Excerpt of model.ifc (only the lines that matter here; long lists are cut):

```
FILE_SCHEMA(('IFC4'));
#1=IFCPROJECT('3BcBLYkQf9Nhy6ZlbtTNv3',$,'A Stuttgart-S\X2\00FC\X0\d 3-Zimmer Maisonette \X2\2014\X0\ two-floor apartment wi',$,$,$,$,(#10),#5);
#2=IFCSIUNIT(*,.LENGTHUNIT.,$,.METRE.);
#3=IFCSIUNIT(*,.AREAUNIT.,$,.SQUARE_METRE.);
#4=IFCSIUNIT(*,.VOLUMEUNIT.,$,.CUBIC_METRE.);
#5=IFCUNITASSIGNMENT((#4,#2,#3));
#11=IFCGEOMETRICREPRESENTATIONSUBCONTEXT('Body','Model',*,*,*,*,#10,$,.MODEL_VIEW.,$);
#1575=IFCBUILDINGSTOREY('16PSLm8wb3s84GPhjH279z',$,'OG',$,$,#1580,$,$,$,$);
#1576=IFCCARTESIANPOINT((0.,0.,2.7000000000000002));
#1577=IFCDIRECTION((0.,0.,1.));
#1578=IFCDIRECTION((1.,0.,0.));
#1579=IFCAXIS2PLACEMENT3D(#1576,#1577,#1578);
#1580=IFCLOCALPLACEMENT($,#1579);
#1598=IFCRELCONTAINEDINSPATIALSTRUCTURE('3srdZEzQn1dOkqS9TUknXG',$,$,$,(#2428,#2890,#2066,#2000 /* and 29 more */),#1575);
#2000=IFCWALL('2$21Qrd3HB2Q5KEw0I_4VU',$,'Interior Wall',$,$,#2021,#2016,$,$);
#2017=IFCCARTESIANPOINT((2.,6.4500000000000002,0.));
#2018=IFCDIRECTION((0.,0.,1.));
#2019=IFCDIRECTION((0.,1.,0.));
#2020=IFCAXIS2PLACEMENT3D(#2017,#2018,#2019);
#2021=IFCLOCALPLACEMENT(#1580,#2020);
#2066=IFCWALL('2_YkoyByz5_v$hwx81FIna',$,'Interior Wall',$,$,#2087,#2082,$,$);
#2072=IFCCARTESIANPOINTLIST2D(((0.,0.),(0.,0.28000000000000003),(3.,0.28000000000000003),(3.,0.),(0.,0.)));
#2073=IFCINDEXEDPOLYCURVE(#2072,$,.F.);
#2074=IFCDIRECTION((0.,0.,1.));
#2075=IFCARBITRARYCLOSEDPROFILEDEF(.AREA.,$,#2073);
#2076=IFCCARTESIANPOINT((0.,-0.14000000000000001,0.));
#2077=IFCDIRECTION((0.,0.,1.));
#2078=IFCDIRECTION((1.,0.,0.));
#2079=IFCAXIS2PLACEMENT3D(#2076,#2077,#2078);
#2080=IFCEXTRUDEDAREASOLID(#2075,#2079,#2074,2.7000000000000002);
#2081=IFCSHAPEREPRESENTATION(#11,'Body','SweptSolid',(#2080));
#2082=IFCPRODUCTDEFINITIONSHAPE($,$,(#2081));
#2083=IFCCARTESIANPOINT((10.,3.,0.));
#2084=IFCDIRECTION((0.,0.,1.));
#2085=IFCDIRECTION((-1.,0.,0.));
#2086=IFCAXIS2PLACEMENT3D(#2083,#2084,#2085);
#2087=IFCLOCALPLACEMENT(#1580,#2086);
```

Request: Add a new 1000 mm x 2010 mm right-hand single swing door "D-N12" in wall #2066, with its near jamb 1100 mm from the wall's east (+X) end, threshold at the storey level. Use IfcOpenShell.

```python
import numpy as np
import ifcopenshell
import ifcopenshell.api.feature
import ifcopenshell.api.geometry
import ifcopenshell.api.root
import ifcopenshell.api.spatial
import ifcopenshell.geom
import ifcopenshell.util.element
import ifcopenshell.util.placement
import ifcopenshell.util.representation
import ifcopenshell.util.shape
import ifcopenshell.util.unit

model = ifcopenshell.open("model.ifc")
unit_scale = ifcopenshell.util.unit.calculate_unit_scale(model)
settings = ifcopenshell.geom.settings()


def volume(element):
    """Net volume in cubic metres, openings subtracted."""
    shape = ifcopenshell.geom.create_shape(settings, element)
    return ifcopenshell.util.shape.get_volume(shape.geometry)


wall = model.by_id(2066)
storey = ifcopenshell.util.element.get_container(wall, ifc_class="IfcBuildingStorey")
context = ifcopenshell.util.representation.get_context(model, "Model", "Body", "MODEL_VIEW")
before = volume(wall)

width, height, from_end, sill = 1, 2.01, 1.1, 0.0  # metres

# The wall runs along its own X axis, and the end named is its -X end.
wall_shape = ifcopenshell.geom.create_shape(settings, wall)
x, y, z = ifcopenshell.util.shape.get_vertices(wall_shape.geometry).T
start = x.min() + from_end
face, thickness = float(y.min()), float(y.max() - y.min())
wall_matrix = ifcopenshell.util.placement.get_local_placement(wall.ObjectPlacement)
level = ifcopenshell.util.placement.get_local_placement(storey.ObjectPlacement)[2, 3]


def in_wall(x, y):
    """Placement at x, y metres in the wall's axes, at sill height."""
    matrix = wall_matrix.copy()
    matrix[:, 3] = wall_matrix @ np.array([x / unit_scale, y / unit_scale, 0.0, 1.0])
    matrix[2, 3] = level + sill / unit_scale
    return matrix


# Opening: a box that overshoots both wall faces by 50 mm.
opening = ifcopenshell.api.root.create_entity(model, ifc_class="IfcOpeningElement", predefined_type="OPENING")
box = ifcopenshell.api.geometry.add_wall_representation(
    model, context=context, length=width, height=height, thickness=thickness + 0.1
)
ifcopenshell.api.geometry.assign_representation(model, product=opening, representation=box)
ifcopenshell.api.geometry.edit_object_placement(model, product=opening, matrix=in_wall(start, face - 0.05), is_si=False)
ifcopenshell.api.feature.add_feature(model, feature=opening, element=wall)

door = ifcopenshell.api.root.create_entity(model, ifc_class="IfcDoor", name="D-N12", predefined_type="DOOR")
door.OverallWidth, door.OverallHeight = width / unit_scale, height / unit_scale
door.OperationType = "SINGLE_SWING_RIGHT"
body = ifcopenshell.api.geometry.add_door_representation(
    model,
    context=context,
    overall_width=door.OverallWidth,
    overall_height=door.OverallHeight,
    operation_type="SINGLE_SWING_RIGHT",
    lining_properties={"LiningDepth": thickness / unit_scale, "ThresholdDepth": thickness / unit_scale},
)
ifcopenshell.api.geometry.assign_representation(model, product=door, representation=body)
ifcopenshell.api.spatial.assign_container(model, products=[door], relating_structure=storey)
ifcopenshell.api.feature.add_filling(model, opening=opening, element=door)

# The lining spans the wall, so the door starts at the wall face.
ifcopenshell.api.geometry.edit_object_placement(model, product=door, matrix=in_wall(start, face), is_si=False)

after = volume(wall)

print(f"wall volume {before:.3f} -> {after:.3f} m3")

model.write("model_rev.ifc")
```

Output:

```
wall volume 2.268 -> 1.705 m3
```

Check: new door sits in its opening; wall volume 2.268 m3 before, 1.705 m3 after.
